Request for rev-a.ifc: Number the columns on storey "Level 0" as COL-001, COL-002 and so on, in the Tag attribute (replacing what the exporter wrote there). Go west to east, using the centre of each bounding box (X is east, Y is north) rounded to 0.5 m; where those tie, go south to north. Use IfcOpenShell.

First a look at what the model holds.

```python
import ifcopenshell
import ifcopenshell.util.element
import ifcopenshell.util.placement

model = ifcopenshell.open("rev-a.ifc")
print(model.schema)
storey = next(s for s in model.by_type("IfcBuildingStorey") if s.Name == "Level 0")
columns = [e for e in ifcopenshell.util.element.get_decomposition(storey) if e.is_a("IfcColumn")]
for e in sorted(columns, key=lambda e: e.id()):
    origin = ifcopenshell.util.placement.get_local_placement(e.ObjectPlacement)[:3, 3]
    print(e.id(), e.Tag, e.Name, origin.round(2) + 0.0, sep=" | ")
```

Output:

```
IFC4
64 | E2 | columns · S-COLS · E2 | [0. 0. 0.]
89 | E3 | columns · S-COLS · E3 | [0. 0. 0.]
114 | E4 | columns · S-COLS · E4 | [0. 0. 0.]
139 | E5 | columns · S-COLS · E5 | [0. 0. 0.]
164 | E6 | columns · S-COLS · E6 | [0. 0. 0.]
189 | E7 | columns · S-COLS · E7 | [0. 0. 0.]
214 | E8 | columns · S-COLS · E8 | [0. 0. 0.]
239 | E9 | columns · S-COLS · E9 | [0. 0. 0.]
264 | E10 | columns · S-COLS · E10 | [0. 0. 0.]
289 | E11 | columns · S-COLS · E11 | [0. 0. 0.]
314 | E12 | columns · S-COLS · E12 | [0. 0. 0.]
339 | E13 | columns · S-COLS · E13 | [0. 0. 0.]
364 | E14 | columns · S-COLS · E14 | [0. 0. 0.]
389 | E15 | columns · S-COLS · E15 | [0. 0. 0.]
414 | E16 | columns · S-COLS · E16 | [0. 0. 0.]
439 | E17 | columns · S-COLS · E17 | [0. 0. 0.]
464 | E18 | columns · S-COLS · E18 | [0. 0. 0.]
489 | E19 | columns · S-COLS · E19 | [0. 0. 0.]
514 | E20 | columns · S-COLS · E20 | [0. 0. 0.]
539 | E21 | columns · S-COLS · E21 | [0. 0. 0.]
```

```python
import ifcopenshell
import ifcopenshell.geom
import ifcopenshell.util.element
import ifcopenshell.util.shape

model = ifcopenshell.open("rev-a.ifc")
settings = ifcopenshell.geom.settings()
settings.set("use-world-coords", True)


def centre(element):
    shape = ifcopenshell.geom.create_shape(settings, element)
    return ifcopenshell.util.shape.get_bbox_centroid(shape.geometry)


storey = next(s for s in model.by_type("IfcBuildingStorey") if s.Name == "Level 0")
columns = [e for e in ifcopenshell.util.element.get_decomposition(storey) if e.is_a("IfcColumn")]

# Insertion points can sit at a corner or the storey origin, so sort by the geometry (in metres).
centres = {e: centre(e) for e in columns}
columns.sort(key=lambda e: (round(centres[e][0] / 0.5), centres[e][1]))

for i, e in enumerate(columns, start=1):
    number = f"COL-0{i:02d}"
    e.Tag = number
    print(e.id(), number)

model.write("rev-a_edited.ifc")
```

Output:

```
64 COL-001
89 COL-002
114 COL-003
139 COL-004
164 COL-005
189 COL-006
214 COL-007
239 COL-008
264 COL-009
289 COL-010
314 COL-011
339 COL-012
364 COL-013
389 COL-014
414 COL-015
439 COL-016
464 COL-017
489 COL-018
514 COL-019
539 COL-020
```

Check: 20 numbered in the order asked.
